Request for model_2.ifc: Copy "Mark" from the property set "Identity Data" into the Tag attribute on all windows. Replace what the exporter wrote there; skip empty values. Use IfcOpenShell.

First a look at what the model holds.

```python
import ifcopenshell
import ifcopenshell.util.element

model = ifcopenshell.open("model_2.ifc")
print(model.schema)
windows = model.by_type("IfcWindow")
print(len(windows), "windows")
for e in windows[:8]:
    source = ifcopenshell.util.element.get_pset(e, "Identity Data", "Mark")
    target = e.Tag
    print(e.id(), repr(source), repr(target), sep=" | ")
```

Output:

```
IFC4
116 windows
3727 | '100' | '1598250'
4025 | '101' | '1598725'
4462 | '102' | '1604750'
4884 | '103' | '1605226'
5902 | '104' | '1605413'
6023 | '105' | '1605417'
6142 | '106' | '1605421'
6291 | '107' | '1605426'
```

```python
import ifcopenshell
import ifcopenshell.util.element

model = ifcopenshell.open("model_2.ifc")

count = 0
for e in model.by_type("IfcWindow"):
    value = ifcopenshell.util.element.get_pset(e, "Identity Data", "Mark")
    current = e.Tag
    if not value or not value.strip() or current == value:
        continue
    e.Tag = value
    count += 1

print(count, "windows updated")

model.write("model_2_updated.ifc")
```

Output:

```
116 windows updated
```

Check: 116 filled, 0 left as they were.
